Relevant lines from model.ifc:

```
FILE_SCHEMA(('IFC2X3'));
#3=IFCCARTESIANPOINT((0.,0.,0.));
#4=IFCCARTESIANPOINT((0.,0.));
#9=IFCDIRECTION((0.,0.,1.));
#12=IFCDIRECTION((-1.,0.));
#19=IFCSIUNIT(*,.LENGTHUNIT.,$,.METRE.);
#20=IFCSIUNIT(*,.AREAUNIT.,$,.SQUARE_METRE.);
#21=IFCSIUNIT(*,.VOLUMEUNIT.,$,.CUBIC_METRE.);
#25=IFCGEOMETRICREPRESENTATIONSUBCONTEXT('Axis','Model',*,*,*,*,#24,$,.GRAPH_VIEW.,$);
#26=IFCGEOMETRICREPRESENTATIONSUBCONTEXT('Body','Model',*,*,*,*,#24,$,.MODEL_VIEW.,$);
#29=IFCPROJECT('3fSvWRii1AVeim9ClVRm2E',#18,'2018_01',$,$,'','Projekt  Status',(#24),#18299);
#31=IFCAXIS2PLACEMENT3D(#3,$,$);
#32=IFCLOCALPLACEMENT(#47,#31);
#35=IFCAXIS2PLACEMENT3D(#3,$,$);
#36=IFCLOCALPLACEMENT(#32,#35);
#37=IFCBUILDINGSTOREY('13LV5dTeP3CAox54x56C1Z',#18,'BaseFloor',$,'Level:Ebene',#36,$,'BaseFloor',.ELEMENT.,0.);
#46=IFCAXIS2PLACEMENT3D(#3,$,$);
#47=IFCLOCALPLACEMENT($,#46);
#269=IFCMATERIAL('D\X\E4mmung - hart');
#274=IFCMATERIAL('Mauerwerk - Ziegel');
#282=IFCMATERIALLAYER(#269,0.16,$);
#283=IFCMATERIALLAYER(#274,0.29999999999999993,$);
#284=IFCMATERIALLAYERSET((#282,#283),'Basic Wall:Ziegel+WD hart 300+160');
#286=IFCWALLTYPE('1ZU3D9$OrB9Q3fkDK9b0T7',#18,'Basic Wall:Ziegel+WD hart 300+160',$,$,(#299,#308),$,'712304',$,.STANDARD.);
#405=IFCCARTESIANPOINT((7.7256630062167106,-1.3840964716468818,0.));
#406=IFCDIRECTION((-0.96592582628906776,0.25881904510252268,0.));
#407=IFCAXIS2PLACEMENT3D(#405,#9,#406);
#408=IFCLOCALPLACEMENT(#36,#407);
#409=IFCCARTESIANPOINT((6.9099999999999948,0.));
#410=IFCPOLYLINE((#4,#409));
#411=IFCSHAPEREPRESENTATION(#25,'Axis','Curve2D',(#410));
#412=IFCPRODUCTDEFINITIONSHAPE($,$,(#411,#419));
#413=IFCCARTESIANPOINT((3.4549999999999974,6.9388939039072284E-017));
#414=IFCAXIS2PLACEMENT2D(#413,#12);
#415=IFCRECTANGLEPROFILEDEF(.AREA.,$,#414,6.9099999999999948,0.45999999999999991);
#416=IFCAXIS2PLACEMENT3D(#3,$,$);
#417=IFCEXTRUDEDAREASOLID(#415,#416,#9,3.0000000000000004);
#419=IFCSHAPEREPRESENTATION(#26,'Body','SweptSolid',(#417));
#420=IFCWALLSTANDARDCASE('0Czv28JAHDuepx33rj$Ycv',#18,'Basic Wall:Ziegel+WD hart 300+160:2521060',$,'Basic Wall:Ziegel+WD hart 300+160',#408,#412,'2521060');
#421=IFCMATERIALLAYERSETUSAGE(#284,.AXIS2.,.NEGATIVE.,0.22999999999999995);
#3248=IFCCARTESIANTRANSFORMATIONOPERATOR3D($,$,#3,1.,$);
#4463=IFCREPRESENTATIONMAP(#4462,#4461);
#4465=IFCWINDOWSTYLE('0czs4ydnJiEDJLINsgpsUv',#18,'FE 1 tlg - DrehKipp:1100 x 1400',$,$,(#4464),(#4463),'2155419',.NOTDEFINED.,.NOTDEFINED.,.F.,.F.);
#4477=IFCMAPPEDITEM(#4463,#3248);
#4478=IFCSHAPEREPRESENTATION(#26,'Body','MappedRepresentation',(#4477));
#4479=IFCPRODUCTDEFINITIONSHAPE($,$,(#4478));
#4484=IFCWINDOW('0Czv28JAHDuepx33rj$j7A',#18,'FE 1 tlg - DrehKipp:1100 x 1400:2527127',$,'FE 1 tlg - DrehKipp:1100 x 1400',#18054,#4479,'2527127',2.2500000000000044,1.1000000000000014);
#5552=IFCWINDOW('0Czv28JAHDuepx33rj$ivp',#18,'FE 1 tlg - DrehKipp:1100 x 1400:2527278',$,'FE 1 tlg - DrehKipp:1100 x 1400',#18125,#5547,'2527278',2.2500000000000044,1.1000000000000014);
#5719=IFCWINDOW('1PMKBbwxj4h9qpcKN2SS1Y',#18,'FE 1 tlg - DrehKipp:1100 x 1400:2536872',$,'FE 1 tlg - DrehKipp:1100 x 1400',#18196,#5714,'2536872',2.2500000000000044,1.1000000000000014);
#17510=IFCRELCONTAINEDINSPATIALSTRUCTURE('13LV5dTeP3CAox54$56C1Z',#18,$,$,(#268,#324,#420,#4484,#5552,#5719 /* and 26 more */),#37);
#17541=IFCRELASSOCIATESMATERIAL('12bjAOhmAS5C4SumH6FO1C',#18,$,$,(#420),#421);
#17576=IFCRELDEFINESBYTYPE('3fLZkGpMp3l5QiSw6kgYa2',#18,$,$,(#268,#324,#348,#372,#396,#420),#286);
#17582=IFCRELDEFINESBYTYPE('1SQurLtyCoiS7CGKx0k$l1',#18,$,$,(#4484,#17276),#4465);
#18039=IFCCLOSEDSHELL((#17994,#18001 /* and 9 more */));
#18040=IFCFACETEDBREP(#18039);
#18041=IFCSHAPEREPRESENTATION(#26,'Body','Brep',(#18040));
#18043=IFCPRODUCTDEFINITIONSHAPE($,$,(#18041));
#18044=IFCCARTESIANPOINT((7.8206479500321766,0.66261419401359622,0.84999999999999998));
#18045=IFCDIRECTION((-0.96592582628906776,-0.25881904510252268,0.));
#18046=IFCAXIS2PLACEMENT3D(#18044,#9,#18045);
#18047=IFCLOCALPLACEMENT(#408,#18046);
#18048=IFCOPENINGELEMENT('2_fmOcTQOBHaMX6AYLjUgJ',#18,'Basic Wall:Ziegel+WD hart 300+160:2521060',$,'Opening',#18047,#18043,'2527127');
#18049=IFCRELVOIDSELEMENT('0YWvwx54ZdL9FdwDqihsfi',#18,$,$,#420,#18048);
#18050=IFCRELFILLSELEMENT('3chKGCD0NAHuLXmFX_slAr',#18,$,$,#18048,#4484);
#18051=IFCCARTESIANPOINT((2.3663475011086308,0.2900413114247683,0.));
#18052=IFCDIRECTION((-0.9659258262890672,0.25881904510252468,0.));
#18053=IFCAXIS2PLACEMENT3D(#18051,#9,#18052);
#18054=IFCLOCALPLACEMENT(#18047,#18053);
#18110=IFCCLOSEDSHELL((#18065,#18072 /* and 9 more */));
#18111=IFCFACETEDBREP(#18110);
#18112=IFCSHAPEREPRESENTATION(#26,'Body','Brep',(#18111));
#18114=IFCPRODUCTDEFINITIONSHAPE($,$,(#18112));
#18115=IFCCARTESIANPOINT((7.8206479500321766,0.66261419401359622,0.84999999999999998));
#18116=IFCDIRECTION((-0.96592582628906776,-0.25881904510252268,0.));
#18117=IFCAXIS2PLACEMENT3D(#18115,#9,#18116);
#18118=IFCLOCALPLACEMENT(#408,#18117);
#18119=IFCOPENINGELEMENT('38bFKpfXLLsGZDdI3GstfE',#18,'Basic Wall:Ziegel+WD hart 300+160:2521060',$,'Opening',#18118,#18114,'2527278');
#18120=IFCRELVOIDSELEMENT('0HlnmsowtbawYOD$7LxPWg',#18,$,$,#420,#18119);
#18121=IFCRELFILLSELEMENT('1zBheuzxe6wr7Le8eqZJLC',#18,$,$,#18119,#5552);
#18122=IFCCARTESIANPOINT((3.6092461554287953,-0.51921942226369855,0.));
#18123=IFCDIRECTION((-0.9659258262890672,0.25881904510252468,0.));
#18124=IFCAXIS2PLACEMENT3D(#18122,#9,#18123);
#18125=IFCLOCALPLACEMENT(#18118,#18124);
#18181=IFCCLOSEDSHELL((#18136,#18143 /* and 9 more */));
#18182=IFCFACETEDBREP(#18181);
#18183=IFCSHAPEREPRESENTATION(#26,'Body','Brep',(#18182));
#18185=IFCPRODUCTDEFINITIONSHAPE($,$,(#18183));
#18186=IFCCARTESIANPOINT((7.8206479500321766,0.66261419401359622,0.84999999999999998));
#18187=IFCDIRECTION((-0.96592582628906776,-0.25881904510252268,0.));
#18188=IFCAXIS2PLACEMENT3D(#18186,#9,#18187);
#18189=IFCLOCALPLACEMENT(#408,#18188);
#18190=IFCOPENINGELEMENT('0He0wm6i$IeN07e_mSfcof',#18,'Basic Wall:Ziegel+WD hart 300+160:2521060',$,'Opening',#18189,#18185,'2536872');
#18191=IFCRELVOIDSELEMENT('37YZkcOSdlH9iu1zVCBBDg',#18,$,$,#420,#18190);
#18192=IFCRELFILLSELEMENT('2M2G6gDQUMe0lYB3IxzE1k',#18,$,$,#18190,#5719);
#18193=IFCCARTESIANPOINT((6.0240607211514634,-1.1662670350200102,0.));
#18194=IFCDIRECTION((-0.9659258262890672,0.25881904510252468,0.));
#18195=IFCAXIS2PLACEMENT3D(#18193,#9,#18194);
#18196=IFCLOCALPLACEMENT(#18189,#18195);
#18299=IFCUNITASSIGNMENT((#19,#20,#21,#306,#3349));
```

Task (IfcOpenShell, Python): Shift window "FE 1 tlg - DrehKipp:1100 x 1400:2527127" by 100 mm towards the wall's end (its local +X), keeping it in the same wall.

```python
import ifcopenshell
import ifcopenshell.api.geometry
import ifcopenshell.util.placement

model = ifcopenshell.open("model.ifc")

window = model.by_guid("0Czv28JAHDuepx33rj$j7A")
opening = window.FillsVoids[0].RelatingOpeningElement
wall = opening.VoidsElements[0].RelatingBuildingElement

wall_matrix = ifcopenshell.util.placement.get_local_placement(wall.ObjectPlacement)
shift = wall_matrix[:3, 0] * 0.1
before = ifcopenshell.util.placement.get_local_placement(window.ObjectPlacement)[:3, 3].copy()

# The window is placed relative to its opening, so it follows when the opening moves.
matrix = ifcopenshell.util.placement.get_local_placement(opening.ObjectPlacement)
matrix[:3, 3] += shift
ifcopenshell.api.geometry.edit_object_placement(
    model, product=opening, matrix=matrix, is_si=False, should_transform_children=True
)

after = ifcopenshell.util.placement.get_local_placement(window.ObjectPlacement)[:3, 3]
print("window moved by", (after - before).round(3) + 0.0)

model.write("model_rev.ifc")
```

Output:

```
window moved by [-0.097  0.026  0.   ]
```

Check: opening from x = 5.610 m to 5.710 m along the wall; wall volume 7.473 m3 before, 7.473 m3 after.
